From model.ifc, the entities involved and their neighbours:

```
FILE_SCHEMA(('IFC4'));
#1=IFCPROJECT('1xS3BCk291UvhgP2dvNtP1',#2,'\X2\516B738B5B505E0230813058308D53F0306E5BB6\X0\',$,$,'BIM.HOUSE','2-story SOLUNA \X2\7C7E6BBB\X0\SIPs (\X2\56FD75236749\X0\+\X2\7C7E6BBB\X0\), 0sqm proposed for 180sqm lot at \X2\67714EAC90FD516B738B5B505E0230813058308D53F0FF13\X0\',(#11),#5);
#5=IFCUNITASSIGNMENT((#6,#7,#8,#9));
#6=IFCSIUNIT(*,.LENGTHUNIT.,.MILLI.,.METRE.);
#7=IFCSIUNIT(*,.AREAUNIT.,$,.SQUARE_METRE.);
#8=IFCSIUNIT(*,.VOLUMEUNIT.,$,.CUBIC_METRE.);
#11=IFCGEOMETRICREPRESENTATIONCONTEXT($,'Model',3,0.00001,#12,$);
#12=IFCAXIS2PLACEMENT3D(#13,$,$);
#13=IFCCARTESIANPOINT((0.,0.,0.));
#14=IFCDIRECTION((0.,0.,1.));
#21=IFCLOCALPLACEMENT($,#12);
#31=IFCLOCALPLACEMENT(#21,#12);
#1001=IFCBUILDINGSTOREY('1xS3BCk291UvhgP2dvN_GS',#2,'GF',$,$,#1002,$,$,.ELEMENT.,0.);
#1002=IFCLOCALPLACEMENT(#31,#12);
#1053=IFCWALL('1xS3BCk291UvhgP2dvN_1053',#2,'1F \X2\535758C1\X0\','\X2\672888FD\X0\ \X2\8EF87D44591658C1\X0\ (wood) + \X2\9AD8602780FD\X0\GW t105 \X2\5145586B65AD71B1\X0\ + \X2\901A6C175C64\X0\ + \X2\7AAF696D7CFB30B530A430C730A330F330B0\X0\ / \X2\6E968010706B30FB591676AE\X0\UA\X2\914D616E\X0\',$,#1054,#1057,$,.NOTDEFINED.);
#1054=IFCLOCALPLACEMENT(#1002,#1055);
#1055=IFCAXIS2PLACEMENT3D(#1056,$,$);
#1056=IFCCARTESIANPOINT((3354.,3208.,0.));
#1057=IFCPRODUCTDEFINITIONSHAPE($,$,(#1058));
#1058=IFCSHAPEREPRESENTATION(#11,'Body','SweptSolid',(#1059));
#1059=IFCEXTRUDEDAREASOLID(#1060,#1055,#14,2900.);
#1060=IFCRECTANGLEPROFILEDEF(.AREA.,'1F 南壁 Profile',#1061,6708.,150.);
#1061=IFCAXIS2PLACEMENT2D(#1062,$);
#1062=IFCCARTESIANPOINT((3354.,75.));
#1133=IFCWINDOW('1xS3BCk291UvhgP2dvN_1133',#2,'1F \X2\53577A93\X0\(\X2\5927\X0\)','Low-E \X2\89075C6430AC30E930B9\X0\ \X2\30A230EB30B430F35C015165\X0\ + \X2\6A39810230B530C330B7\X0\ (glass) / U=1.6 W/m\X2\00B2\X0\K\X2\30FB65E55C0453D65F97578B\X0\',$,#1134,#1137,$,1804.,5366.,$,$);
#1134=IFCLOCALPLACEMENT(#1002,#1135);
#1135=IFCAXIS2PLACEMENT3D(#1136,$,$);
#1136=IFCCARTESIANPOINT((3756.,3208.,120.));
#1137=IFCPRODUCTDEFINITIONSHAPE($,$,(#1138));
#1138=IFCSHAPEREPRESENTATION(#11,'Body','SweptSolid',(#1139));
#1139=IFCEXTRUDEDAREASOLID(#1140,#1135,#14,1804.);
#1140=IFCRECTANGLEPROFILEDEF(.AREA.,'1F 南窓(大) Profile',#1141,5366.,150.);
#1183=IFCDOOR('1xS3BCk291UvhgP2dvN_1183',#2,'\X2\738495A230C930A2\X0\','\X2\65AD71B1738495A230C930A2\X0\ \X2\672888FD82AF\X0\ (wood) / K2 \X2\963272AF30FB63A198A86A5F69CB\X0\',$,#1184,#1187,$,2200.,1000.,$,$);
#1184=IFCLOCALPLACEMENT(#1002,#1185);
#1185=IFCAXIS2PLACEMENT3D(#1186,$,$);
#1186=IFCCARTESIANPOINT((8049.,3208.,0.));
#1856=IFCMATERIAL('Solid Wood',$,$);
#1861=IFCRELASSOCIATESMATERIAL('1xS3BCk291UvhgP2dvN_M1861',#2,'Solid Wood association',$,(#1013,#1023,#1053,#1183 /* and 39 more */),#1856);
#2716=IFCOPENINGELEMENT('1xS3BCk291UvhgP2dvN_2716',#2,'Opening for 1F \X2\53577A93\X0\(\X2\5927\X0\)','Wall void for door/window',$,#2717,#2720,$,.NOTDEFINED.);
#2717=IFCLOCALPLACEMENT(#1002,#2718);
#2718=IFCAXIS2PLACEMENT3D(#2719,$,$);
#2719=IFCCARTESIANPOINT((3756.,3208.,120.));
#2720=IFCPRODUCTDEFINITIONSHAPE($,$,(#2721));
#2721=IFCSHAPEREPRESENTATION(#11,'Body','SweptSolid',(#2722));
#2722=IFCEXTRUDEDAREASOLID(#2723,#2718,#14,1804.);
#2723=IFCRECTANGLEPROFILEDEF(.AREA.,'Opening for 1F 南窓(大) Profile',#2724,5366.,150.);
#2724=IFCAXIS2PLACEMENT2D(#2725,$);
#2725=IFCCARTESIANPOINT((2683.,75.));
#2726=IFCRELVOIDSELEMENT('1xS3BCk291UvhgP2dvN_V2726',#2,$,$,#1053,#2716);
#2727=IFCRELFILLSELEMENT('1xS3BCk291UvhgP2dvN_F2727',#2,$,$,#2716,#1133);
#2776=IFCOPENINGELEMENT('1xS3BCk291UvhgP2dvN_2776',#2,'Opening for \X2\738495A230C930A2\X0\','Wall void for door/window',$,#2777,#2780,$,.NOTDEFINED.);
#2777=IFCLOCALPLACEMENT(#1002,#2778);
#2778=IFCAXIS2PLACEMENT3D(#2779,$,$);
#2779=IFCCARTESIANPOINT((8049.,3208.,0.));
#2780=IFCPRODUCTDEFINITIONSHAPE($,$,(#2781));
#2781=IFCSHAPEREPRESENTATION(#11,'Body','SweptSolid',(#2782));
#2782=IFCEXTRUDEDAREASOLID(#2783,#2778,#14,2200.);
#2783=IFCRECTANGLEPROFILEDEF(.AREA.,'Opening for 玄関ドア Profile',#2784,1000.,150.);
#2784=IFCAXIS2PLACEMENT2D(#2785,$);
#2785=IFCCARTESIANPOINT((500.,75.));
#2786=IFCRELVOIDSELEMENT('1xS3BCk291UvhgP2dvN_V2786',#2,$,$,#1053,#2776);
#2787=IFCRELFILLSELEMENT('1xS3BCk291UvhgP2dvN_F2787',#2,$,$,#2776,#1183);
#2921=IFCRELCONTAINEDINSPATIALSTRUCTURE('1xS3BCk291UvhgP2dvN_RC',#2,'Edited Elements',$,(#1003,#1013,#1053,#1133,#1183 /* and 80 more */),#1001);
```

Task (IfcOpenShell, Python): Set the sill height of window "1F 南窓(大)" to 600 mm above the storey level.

```python
import numpy as np
import ifcopenshell
import ifcopenshell.api.geometry
import ifcopenshell.geom
import ifcopenshell.util.element
import ifcopenshell.util.placement
import ifcopenshell.util.shape
import ifcopenshell.util.unit

model = ifcopenshell.open("model.ifc")
unit_scale = ifcopenshell.util.unit.calculate_unit_scale(model)

window = model.by_id(1133)
opening = window.FillsVoids[0].RelatingOpeningElement
storey = ifcopenshell.util.element.get_container(window, ifc_class="IfcBuildingStorey")
level = ifcopenshell.util.placement.get_local_placement(storey.ObjectPlacement)[2, 3]

# The opening's origin need not be at the sill, so measure its lowest point.
shape = ifcopenshell.geom.create_shape(ifcopenshell.geom.settings(), opening)
bottom = ifcopenshell.util.shape.get_shape_bottom_elevation(shape, shape.geometry) / unit_scale
dz = level + 0.6 / unit_scale - bottom

shift = np.array([0.0, 0.0, dz])
# The window is not placed relative to its opening, so move both.
for product in (opening, window):
    matrix = ifcopenshell.util.placement.get_local_placement(product.ObjectPlacement)
    matrix[:3, 3] += shift
    ifcopenshell.api.geometry.edit_object_placement(model, product=product, matrix=matrix, is_si=False)

print(f"moved by {dz * unit_scale:+.3f} m")

model.write("model_rev.ifc")
```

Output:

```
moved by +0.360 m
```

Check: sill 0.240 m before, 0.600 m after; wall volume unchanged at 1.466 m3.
